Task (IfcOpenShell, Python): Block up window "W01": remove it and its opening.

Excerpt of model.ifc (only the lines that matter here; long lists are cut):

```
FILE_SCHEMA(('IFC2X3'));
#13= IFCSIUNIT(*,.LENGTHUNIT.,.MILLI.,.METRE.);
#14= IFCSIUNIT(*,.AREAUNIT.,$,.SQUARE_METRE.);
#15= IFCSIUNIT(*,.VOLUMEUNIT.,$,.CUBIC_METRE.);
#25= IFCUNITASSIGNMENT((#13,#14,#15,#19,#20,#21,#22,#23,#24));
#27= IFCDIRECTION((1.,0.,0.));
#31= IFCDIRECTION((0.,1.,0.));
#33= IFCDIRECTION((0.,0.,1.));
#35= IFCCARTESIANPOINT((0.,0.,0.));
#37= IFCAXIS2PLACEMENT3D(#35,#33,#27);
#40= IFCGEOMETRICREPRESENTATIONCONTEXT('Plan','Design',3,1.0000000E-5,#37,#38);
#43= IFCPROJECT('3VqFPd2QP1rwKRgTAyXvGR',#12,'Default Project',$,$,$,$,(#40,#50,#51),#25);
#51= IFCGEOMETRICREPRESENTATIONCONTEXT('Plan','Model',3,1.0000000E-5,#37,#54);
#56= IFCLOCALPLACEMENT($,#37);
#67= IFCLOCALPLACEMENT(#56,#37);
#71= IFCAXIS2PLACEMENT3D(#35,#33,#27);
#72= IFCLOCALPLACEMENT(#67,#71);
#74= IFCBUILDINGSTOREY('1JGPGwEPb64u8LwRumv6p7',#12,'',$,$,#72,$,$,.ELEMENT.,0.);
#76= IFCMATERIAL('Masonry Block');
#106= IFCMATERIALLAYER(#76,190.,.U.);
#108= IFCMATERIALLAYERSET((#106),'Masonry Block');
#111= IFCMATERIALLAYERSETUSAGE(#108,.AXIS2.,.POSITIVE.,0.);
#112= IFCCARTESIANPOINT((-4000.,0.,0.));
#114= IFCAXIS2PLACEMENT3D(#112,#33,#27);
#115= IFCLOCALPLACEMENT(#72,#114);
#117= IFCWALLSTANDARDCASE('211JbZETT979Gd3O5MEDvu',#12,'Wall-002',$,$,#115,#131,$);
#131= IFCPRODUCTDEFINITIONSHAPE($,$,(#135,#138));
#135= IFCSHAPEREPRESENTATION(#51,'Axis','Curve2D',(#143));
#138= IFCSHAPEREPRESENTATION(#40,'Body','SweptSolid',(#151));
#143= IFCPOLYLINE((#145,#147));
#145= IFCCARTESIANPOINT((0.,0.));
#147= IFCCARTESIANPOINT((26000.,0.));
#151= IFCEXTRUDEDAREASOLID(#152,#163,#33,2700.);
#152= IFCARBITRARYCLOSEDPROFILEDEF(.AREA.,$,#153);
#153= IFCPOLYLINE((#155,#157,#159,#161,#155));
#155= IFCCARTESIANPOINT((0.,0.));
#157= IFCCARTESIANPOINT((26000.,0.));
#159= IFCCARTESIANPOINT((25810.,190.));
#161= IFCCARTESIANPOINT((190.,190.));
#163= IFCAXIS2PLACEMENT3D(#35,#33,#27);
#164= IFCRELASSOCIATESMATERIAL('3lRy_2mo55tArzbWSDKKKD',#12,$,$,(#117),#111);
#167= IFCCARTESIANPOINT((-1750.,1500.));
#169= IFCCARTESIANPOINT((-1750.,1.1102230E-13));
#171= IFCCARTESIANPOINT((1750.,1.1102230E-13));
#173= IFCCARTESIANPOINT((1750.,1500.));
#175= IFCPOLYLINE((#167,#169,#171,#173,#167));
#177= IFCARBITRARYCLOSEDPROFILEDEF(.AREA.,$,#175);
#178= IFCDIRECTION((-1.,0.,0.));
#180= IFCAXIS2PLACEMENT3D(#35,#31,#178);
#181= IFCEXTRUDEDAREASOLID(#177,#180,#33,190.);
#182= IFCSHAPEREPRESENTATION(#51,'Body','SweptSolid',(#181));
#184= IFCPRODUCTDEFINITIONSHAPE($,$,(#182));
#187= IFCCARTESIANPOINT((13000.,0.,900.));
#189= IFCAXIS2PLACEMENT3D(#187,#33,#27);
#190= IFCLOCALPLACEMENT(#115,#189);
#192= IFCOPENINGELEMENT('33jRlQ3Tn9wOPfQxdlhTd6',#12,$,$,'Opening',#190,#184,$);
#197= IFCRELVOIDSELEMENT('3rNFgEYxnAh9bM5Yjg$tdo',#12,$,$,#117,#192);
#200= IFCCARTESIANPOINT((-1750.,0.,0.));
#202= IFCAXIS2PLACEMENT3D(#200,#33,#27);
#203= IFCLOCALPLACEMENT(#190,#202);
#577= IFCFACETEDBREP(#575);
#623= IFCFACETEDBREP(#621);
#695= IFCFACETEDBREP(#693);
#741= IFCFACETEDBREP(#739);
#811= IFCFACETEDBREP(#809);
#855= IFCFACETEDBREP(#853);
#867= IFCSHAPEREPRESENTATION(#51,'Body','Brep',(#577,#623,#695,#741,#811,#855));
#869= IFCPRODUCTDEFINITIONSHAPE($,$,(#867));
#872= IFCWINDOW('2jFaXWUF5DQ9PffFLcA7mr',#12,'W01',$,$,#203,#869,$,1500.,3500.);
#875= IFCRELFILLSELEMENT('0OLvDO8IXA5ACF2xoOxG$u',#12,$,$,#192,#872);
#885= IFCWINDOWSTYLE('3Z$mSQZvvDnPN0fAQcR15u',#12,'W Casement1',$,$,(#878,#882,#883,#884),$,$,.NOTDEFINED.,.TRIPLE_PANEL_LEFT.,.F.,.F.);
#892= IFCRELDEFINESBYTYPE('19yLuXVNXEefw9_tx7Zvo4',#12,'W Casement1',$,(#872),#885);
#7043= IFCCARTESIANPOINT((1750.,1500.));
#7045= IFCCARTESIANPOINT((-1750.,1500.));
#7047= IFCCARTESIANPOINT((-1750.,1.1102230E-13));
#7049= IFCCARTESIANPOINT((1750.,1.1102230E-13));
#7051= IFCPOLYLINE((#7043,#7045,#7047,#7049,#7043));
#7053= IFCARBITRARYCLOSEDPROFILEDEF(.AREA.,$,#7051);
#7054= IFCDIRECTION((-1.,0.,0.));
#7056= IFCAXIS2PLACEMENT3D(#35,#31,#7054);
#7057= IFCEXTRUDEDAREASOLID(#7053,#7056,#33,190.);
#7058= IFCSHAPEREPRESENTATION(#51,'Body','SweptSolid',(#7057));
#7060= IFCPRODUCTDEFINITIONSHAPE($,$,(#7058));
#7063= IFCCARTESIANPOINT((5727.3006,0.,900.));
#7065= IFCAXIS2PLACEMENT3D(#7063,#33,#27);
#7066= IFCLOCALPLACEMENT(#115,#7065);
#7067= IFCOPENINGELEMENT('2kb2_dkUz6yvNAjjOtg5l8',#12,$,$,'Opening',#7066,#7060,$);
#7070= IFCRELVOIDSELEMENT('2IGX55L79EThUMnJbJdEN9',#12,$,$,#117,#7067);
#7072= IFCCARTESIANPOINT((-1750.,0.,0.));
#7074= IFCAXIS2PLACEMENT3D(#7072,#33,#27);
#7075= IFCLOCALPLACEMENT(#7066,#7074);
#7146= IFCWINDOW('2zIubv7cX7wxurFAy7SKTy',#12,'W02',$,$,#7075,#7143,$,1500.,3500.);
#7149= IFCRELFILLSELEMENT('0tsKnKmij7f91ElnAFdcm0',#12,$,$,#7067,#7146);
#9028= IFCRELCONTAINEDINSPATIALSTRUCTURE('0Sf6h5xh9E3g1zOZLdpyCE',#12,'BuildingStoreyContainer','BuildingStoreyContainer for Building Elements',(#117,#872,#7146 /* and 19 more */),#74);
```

```python
import ifcopenshell
import ifcopenshell.api.feature
import ifcopenshell.api.root
import ifcopenshell.geom
import ifcopenshell.util.shape

model = ifcopenshell.open("model.ifc")
settings = ifcopenshell.geom.settings()


def volume(element):
    """Net volume in cubic metres, openings subtracted."""
    shape = ifcopenshell.geom.create_shape(settings, element)
    return ifcopenshell.util.shape.get_volume(shape.geometry)


window = model.by_id(872)
opening = window.FillsVoids[0].RelatingOpeningElement
wall = opening.VoidsElements[0].RelatingBuildingElement
before = volume(wall)

ifcopenshell.api.root.remove_product(model, product=window)
ifcopenshell.api.feature.remove_feature(model, feature=opening)

after = volume(wall)

print(f"wall volume {before:.3f} -> {after:.3f} m3")

model.write("model_rev.ifc")
```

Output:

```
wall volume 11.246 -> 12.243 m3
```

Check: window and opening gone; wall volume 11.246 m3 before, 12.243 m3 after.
